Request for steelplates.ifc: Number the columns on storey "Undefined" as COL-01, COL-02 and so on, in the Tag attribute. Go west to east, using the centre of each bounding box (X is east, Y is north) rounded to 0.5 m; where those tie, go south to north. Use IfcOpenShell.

First a look at what the model holds.

```python
import ifcopenshell
import ifcopenshell.util.element
import ifcopenshell.util.placement

model = ifcopenshell.open("steelplates.ifc")
print(model.schema)
storey = next(s for s in model.by_type("IfcBuildingStorey") if s.Name == "Undefined")
columns = [e for e in ifcopenshell.util.element.get_decomposition(storey) if e.is_a("IfcColumn")]
for e in sorted(columns, key=lambda e: e.id()):
    origin = ifcopenshell.util.placement.get_local_placement(e.ObjectPlacement)[:3, 3]
    print(e.id(), e.Tag, e.Name, origin.round(2) + 0.0, sep=" | ")
```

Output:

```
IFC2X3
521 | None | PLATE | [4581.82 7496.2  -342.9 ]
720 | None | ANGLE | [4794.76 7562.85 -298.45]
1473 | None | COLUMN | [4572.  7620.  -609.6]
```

```python
import ifcopenshell
import ifcopenshell.geom
import ifcopenshell.util.element
import ifcopenshell.util.shape

model = ifcopenshell.open("steelplates.ifc")
settings = ifcopenshell.geom.settings()
settings.set("use-world-coords", True)


def centre(element):
    shape = ifcopenshell.geom.create_shape(settings, element)
    return ifcopenshell.util.shape.get_bbox_centroid(shape.geometry)


storey = next(s for s in model.by_type("IfcBuildingStorey") if s.Name == "Undefined")
columns = [e for e in ifcopenshell.util.element.get_decomposition(storey) if e.is_a("IfcColumn")]

# Insertion points can sit at a corner or the storey origin, so sort by the geometry (in metres).
centres = {e: centre(e) for e in columns}
columns.sort(key=lambda e: (round(centres[e][0] / 0.5), centres[e][1]))

for i, e in enumerate(columns, start=1):
    number = f"COL-{i:02d}"
    e.Tag = number
    print(e.id(), number)

model.write("steelplates_v2.ifc")
```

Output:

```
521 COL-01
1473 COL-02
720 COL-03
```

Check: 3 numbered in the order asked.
